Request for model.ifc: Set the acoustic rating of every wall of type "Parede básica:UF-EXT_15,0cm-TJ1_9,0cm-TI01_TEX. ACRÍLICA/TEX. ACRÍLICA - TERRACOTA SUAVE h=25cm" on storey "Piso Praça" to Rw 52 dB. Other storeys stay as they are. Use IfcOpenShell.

First a look at what the model holds.

```python
import ifcopenshell
import ifcopenshell.util.element

model = ifcopenshell.open("model.ifc")
print(model.schema)
storey = next(s for s in model.by_type("IfcBuildingStorey") if s.Name == "Piso Praça")
walls = [e for e in ifcopenshell.util.element.get_decomposition(storey) if e.is_a("IfcWall")]
seen = {}
for e in walls:
    element_type = ifcopenshell.util.element.get_type(e)
    key = (element_type.Name if element_type != e and element_type else None, ifcopenshell.util.element.get_pset(e, "Pset_WallCommon", "AcousticRating"))
    seen[key] = seen.get(key, 0) + 1
for (name, value), count in sorted(seen.items(), key=str):
    print(count, "x", name, "|", value)
```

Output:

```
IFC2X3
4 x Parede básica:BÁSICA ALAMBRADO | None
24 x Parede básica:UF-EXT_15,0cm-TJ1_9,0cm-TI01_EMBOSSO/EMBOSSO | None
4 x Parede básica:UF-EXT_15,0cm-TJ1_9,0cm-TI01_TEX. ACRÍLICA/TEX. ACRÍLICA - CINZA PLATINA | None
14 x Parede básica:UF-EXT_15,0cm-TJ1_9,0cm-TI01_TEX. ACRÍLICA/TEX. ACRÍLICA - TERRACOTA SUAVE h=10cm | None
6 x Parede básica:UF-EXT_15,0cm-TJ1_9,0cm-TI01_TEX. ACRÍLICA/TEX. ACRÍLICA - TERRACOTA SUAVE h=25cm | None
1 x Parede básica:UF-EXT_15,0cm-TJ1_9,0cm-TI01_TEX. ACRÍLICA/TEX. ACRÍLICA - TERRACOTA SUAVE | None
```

```python
import ifcopenshell
import ifcopenshell.api.pset
import ifcopenshell.util.element

model = ifcopenshell.open("model.ifc")

storey = next(s for s in model.by_type("IfcBuildingStorey") if s.Name == "Piso Praça")
walls = [e for e in ifcopenshell.util.element.get_decomposition(storey) if e.is_a("IfcWall")]

count = 0
for e in walls:
    element_type = ifcopenshell.util.element.get_type(e)
    if element_type in (None, e) or element_type.Name != "Parede básica:UF-EXT_15,0cm-TJ1_9,0cm-TI01_TEX. ACRÍLICA/TEX. ACRÍLICA - TERRACOTA SUAVE h=25cm":
        continue
    # add_pset returns the element's existing set when there is one.
    pset = ifcopenshell.api.pset.add_pset(model, product=e, name="Pset_WallCommon")
    ifcopenshell.api.pset.edit_pset(model, pset=pset, properties={"AcousticRating": "Rw 52 dB"})
    count += 1

print(count, "walls updated")

model.write("model_rev.ifc")
```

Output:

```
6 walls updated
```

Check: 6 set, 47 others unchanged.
